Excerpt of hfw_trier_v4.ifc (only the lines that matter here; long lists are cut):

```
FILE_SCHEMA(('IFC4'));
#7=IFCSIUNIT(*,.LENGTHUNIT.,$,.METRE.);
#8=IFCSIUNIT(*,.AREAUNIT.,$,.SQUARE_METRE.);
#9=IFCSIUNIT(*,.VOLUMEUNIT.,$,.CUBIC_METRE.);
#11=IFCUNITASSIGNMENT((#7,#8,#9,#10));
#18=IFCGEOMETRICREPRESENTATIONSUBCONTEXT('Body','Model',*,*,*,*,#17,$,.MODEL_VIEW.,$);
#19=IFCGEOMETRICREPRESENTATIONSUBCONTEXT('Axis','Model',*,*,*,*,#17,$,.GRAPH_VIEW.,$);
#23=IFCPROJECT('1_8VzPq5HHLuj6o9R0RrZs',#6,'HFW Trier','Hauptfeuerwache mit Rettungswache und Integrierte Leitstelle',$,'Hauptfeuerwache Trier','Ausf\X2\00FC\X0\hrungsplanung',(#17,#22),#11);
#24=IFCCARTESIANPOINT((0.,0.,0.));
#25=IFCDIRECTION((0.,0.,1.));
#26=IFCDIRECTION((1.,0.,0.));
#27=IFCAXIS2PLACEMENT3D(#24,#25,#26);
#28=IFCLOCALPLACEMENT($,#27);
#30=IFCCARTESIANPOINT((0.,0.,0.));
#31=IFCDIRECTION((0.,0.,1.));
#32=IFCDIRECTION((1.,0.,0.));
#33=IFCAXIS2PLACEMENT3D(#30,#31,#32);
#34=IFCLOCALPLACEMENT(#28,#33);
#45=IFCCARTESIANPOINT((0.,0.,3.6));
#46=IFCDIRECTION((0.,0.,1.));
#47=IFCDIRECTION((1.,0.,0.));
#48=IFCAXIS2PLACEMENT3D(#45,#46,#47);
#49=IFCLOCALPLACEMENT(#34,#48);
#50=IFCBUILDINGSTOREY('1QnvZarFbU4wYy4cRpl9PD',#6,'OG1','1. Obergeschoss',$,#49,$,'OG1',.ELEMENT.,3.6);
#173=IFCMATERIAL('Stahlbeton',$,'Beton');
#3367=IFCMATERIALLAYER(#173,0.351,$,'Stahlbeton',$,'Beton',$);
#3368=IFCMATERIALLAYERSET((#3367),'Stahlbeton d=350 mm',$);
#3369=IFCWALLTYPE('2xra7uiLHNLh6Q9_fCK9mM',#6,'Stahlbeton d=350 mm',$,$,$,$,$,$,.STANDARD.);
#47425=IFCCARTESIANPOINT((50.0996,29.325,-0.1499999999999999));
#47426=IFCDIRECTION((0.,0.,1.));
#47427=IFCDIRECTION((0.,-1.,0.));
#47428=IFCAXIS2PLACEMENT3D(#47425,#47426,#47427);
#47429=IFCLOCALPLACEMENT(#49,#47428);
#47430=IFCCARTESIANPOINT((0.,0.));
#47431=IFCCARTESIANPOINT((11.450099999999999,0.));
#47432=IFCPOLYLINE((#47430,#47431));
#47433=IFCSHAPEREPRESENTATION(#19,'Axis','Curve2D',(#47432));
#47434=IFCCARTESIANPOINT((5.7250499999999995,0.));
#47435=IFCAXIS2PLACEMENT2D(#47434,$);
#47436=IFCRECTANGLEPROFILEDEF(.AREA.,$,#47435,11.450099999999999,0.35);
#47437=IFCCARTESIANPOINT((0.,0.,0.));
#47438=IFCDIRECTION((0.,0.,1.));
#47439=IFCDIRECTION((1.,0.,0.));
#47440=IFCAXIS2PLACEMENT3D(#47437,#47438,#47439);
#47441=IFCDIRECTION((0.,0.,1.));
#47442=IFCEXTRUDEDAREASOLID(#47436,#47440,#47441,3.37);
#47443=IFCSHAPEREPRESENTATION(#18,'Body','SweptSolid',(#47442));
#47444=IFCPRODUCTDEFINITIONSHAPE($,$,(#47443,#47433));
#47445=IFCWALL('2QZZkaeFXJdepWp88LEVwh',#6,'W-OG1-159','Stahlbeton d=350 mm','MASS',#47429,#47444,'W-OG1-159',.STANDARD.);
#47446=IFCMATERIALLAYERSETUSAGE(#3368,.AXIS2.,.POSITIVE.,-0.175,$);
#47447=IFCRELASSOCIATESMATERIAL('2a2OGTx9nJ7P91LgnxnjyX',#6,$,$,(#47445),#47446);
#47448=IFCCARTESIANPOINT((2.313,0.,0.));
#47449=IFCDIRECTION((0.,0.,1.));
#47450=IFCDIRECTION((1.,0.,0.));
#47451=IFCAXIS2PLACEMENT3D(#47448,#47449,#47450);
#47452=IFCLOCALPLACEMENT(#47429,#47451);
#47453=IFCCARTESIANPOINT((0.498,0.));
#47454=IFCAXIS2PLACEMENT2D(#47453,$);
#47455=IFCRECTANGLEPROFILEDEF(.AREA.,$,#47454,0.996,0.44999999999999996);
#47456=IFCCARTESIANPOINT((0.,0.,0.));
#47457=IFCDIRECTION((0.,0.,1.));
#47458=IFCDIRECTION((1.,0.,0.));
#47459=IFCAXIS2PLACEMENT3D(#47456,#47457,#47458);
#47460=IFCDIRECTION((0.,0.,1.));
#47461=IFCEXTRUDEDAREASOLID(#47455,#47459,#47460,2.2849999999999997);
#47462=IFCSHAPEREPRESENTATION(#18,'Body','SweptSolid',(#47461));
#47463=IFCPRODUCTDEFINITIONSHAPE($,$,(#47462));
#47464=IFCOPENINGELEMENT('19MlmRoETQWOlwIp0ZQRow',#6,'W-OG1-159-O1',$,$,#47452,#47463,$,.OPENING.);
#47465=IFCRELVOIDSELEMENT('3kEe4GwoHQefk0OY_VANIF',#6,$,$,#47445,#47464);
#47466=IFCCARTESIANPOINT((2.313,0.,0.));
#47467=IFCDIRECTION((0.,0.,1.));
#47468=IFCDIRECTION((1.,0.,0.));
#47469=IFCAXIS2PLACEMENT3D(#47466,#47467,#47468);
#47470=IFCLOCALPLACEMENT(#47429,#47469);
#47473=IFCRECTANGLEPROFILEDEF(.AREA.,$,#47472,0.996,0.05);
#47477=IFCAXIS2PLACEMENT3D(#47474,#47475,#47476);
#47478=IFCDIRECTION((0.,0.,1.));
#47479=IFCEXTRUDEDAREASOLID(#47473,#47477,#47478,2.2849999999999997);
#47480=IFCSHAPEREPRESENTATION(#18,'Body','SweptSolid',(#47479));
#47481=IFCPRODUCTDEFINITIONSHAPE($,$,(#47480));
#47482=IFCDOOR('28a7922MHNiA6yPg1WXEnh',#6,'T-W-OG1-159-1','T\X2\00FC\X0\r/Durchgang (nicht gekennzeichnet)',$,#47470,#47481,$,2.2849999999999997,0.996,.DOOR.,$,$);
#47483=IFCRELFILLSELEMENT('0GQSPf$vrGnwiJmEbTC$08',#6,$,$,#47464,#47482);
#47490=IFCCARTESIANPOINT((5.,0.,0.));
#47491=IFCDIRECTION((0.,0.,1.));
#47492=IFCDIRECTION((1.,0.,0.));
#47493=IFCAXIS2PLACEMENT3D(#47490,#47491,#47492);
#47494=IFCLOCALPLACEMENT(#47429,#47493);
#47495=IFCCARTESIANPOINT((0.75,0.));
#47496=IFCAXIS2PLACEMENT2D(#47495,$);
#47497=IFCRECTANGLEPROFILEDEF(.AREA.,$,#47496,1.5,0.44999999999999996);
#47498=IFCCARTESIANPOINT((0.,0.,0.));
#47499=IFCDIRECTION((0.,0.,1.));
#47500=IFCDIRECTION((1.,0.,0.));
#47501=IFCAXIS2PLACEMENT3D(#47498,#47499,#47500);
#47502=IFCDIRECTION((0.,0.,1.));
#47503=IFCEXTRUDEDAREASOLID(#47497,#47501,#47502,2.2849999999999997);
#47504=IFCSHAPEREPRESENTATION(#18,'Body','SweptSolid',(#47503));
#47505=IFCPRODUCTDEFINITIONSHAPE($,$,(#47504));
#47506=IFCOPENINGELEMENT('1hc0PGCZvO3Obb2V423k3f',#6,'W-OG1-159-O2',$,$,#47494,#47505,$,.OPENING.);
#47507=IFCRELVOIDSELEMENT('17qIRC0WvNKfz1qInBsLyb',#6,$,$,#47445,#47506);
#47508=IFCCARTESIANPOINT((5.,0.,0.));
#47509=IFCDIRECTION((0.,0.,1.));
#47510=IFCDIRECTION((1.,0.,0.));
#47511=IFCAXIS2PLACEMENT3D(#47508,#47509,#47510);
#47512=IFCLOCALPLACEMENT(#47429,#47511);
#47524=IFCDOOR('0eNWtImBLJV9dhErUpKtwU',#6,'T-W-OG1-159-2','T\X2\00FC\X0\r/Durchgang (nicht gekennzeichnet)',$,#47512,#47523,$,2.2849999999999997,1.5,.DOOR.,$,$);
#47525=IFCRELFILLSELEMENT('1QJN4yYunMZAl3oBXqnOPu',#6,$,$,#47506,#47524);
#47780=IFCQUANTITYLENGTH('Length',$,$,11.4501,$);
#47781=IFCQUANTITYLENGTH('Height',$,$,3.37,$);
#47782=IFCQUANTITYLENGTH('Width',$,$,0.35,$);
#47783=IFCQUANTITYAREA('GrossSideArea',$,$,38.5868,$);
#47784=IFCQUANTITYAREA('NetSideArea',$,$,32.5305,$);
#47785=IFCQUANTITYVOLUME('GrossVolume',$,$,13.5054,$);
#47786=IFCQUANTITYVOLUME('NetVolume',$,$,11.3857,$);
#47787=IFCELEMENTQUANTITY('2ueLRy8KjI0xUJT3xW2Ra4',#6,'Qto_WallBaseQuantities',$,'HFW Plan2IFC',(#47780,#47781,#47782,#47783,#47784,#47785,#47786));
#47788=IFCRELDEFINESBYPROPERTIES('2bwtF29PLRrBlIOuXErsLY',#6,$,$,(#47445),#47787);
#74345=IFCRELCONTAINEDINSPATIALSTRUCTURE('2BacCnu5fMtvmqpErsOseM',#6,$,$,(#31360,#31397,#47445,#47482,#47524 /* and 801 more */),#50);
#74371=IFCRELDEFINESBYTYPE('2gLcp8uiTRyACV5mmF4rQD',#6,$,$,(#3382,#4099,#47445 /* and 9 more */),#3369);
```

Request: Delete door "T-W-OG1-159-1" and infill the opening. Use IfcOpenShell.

```python
import ifcopenshell
import ifcopenshell.api.feature
import ifcopenshell.api.pset
import ifcopenshell.api.root
import ifcopenshell.geom
import ifcopenshell.util.element
import ifcopenshell.util.shape
import ifcopenshell.util.unit

model = ifcopenshell.open("hfw_trier_v4.ifc")
area_scale = ifcopenshell.util.unit.calculate_unit_scale(model, "AREAUNIT")
volume_scale = ifcopenshell.util.unit.calculate_unit_scale(model, "VOLUMEUNIT")
settings = ifcopenshell.geom.settings()


def volume(element):
    """Net volume in cubic metres, openings subtracted."""
    shape = ifcopenshell.geom.create_shape(settings, element)
    return ifcopenshell.util.shape.get_volume(shape.geometry)


door = model.by_id(47482)
opening = door.FillsVoids[0].RelatingOpeningElement
wall = opening.VoidsElements[0].RelatingBuildingElement
before = volume(wall)

ifcopenshell.api.root.remove_product(model, product=door)
ifcopenshell.api.feature.remove_feature(model, feature=opening)

after = volume(wall)
thickness = 0.35  # wall thickness in metres

# Update the wall's stored quantities.
qto = model.by_id(ifcopenshell.util.element.get_pset(wall, "Qto_WallBaseQuantities", should_inherit=False)["id"])
ifcopenshell.api.pset.edit_qto(model, qto=qto, properties={
    "NetSideArea": after / thickness / area_scale,
    "NetVolume": after / volume_scale,
})

print(f"wall volume {before:.3f} -> {after:.3f} m3")

model.write("hfw_trier_v4_updated.ifc")
```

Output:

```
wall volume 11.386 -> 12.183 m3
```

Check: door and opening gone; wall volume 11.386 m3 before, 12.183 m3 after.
